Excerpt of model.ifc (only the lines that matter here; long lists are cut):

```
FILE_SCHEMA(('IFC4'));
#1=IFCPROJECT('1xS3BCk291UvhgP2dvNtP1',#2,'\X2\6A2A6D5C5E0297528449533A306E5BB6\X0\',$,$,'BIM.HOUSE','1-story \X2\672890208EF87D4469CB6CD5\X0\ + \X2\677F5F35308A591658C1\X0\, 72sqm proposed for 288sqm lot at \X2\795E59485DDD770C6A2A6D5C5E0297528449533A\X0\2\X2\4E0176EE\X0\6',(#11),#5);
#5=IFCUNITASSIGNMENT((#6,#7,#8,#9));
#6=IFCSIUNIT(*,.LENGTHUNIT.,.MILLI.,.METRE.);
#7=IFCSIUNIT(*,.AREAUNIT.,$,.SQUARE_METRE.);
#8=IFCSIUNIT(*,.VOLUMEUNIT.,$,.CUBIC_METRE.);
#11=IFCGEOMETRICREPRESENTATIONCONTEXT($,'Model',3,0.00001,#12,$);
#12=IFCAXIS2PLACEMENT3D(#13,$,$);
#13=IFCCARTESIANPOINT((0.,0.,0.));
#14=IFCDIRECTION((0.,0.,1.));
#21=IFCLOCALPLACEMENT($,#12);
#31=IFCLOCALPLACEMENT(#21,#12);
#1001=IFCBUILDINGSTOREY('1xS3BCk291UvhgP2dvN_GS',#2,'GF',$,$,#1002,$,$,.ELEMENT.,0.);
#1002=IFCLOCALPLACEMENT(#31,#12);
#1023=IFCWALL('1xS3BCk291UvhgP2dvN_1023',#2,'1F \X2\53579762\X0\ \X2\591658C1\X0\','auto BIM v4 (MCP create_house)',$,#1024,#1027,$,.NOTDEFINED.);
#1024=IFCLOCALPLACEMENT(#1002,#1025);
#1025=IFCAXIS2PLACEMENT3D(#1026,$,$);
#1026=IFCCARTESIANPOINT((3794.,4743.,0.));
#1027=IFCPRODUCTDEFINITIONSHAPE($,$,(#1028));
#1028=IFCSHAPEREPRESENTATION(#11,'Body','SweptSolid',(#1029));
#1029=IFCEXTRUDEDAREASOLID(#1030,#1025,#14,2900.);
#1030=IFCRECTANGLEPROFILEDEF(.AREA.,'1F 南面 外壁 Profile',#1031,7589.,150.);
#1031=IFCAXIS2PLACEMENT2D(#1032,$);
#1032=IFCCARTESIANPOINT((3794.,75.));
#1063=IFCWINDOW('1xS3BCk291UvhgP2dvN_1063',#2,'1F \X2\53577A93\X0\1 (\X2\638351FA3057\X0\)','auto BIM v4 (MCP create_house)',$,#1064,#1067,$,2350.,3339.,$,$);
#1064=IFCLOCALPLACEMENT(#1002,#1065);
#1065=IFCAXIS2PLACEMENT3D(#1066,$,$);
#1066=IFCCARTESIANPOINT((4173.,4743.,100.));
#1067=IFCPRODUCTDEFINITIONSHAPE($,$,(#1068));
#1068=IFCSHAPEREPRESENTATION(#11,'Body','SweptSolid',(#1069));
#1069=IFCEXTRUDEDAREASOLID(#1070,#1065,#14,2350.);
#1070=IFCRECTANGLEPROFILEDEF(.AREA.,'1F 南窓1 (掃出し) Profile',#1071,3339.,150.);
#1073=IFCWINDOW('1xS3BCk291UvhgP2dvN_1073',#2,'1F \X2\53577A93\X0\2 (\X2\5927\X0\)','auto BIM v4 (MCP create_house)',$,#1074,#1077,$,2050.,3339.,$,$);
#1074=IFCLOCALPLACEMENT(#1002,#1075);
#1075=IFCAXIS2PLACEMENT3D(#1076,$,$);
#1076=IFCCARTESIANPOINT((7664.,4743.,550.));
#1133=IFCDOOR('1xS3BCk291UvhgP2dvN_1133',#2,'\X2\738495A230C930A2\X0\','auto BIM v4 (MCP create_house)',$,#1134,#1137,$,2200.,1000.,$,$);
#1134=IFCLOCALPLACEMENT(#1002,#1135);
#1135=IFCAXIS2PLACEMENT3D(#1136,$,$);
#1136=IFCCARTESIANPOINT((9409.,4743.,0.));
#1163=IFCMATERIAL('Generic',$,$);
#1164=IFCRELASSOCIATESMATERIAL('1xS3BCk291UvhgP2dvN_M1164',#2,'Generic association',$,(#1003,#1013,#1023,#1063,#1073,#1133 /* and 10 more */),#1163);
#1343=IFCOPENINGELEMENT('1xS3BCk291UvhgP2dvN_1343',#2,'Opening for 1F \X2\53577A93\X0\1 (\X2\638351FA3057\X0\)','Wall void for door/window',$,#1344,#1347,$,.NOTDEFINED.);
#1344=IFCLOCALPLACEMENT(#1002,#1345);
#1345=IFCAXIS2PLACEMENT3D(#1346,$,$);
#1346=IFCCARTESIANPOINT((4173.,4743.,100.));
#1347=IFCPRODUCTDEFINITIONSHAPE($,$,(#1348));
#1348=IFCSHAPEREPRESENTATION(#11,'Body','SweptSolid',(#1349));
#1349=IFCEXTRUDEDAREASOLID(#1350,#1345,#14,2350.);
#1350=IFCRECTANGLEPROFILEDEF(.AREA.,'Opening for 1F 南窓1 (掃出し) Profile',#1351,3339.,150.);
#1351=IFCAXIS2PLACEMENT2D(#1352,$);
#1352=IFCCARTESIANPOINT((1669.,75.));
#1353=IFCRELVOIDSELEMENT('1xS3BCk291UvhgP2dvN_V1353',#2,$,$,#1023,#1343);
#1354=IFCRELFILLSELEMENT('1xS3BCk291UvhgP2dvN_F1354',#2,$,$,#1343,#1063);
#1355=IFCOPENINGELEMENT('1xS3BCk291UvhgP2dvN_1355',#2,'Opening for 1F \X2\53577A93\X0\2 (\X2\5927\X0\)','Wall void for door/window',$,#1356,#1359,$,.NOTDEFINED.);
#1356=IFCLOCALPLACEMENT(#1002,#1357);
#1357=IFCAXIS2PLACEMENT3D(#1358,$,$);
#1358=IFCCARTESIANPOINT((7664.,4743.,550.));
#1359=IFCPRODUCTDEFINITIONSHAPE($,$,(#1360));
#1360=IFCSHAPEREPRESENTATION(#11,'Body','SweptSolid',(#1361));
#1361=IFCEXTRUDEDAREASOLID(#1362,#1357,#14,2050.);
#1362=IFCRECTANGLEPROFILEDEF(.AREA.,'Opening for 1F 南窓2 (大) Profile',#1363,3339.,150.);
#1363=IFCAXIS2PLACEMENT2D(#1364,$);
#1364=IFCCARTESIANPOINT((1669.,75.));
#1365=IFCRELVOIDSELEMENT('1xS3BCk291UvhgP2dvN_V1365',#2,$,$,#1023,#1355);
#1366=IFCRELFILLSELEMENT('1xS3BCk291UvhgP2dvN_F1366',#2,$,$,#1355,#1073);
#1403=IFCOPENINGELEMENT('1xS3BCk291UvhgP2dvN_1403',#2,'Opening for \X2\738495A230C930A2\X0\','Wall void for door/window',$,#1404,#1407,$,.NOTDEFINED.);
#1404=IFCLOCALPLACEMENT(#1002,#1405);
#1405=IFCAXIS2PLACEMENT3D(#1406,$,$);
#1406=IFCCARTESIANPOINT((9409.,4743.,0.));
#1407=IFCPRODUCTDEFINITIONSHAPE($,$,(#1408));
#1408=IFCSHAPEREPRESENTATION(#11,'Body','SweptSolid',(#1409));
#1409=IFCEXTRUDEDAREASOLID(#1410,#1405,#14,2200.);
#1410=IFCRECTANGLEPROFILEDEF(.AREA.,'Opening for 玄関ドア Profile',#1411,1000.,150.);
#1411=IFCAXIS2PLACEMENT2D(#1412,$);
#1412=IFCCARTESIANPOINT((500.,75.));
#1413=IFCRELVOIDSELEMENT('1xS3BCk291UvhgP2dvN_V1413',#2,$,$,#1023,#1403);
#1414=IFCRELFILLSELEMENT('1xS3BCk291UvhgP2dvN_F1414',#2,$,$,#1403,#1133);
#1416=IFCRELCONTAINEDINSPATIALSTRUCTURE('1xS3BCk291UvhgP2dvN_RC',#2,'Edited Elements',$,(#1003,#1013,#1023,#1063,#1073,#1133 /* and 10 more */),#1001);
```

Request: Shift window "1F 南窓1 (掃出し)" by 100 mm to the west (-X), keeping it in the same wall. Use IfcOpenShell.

```python
import ifcopenshell
import ifcopenshell.api.geometry
import ifcopenshell.util.placement
import ifcopenshell.util.unit

model = ifcopenshell.open("model.ifc")
unit_scale = ifcopenshell.util.unit.calculate_unit_scale(model)

window = model.by_guid("1xS3BCk291UvhgP2dvN_1063")
opening = window.FillsVoids[0].RelatingOpeningElement
wall = opening.VoidsElements[0].RelatingBuildingElement

wall_matrix = ifcopenshell.util.placement.get_local_placement(wall.ObjectPlacement)
shift = wall_matrix[:3, 0] * -0.1 / unit_scale
before = ifcopenshell.util.placement.get_local_placement(window.ObjectPlacement)[:3, 3].copy()

# The window is not placed relative to its opening, so move both.
for product in (opening, window):
    matrix = ifcopenshell.util.placement.get_local_placement(product.ObjectPlacement)
    matrix[:3, 3] += shift
    ifcopenshell.api.geometry.edit_object_placement(model, product=product, matrix=matrix, is_si=False)

after = ifcopenshell.util.placement.get_local_placement(window.ObjectPlacement)[:3, 3]
print("window moved by", (after - before).round(3) + 0.0)

model.write("model-out.ifc")
```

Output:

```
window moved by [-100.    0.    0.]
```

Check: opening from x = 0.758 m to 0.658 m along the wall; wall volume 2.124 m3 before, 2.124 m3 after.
